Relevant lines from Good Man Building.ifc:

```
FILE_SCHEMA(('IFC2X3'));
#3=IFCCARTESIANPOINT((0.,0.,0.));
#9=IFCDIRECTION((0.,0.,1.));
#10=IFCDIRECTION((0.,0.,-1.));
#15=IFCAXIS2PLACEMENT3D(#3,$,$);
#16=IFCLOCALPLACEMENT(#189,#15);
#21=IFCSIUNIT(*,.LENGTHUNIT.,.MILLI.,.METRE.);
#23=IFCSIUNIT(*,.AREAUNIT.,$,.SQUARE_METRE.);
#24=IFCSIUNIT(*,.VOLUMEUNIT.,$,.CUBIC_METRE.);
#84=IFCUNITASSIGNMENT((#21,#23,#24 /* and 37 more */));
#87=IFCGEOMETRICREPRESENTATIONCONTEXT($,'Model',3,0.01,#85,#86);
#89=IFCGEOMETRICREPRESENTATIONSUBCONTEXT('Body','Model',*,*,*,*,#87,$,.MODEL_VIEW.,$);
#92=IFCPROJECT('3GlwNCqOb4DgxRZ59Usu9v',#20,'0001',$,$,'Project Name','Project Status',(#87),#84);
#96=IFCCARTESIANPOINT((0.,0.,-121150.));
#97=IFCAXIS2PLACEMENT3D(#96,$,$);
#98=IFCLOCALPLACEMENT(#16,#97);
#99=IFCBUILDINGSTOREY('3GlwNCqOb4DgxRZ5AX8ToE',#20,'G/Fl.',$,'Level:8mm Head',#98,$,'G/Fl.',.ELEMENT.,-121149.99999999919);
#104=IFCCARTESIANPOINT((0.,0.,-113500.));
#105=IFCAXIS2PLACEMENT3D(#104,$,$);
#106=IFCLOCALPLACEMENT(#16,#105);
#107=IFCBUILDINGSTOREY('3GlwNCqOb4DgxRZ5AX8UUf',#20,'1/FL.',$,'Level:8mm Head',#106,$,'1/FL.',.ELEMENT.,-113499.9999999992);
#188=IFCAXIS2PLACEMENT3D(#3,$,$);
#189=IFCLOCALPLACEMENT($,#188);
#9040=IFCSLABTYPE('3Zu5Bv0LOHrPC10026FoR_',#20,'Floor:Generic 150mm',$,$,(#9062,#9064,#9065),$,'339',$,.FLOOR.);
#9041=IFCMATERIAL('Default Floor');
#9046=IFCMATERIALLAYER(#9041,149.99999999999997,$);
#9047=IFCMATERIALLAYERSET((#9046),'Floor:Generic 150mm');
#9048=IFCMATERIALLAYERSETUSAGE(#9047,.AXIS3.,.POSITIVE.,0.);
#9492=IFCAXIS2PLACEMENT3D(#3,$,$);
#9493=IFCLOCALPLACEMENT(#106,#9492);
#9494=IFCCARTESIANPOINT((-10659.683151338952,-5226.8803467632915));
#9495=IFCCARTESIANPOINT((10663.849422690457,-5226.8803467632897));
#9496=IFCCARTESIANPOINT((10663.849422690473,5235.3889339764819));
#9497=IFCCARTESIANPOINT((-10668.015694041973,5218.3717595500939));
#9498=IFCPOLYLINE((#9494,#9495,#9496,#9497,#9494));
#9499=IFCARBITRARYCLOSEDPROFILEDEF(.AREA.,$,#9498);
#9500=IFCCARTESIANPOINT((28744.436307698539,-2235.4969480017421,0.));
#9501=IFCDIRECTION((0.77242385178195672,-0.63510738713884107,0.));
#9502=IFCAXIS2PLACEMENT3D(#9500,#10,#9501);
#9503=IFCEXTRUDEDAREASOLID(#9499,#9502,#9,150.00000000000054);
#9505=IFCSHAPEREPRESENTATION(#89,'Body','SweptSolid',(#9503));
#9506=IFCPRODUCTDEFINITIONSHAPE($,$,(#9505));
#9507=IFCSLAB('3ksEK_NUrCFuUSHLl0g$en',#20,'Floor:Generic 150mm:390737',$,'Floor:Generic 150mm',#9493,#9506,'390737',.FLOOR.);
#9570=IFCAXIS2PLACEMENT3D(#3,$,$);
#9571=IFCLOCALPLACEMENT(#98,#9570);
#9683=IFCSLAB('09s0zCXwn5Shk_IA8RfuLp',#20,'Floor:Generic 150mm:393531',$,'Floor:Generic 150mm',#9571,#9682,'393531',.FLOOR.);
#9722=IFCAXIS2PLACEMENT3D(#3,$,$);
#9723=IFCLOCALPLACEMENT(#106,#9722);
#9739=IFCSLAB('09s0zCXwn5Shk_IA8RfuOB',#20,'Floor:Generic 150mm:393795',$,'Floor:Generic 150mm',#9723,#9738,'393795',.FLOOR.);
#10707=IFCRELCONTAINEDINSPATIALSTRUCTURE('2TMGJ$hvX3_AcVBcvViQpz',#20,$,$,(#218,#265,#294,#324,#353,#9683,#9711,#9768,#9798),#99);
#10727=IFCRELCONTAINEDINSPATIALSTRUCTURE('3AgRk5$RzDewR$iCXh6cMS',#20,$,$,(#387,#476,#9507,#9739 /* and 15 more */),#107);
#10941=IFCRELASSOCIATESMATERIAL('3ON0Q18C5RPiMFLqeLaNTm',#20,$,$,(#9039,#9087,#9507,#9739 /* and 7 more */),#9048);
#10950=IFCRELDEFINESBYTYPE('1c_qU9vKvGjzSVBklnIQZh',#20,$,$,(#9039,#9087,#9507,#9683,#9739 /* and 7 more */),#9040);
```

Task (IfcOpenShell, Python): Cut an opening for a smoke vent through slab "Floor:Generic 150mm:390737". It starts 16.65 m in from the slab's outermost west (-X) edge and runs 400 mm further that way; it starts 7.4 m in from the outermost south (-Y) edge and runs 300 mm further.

```python
import numpy as np
import ifcopenshell
import ifcopenshell.api.feature
import ifcopenshell.api.geometry
import ifcopenshell.api.root
import ifcopenshell.geom
import ifcopenshell.util.placement
import ifcopenshell.util.representation
import ifcopenshell.util.shape
import ifcopenshell.util.unit

model = ifcopenshell.open("Good Man Building.ifc")
unit_scale = ifcopenshell.util.unit.calculate_unit_scale(model)
settings = ifcopenshell.geom.settings()


def volume(element):
    """Net volume in cubic metres, openings subtracted."""
    shape = ifcopenshell.geom.create_shape(settings, element)
    return ifcopenshell.util.shape.get_volume(shape.geometry)


slab = model.by_id(9507)
before = volume(slab)

# Extent in the slab's own axes, in metres. The edges named are its -X and -Y sides.
slab_shape = ifcopenshell.geom.create_shape(settings, slab)
vertices = ifcopenshell.util.shape.get_vertices(slab_shape.geometry)
x_min, y_min, bottom = vertices.min(axis=0)
top = vertices[:, 2].max()

opening = ifcopenshell.api.root.create_entity(model, ifc_class="IfcOpeningElement", name="Smoke vent opening")
context = ifcopenshell.util.representation.get_context(model, "Model", "Body", "MODEL_VIEW")
width, depth = 0.4, 0.3
outline = [(0.0, 0.0), (width, 0.0), (width, depth), (0.0, depth), (0.0, 0.0)]
# Overshoot both faces by 50 mm so the cut is clean.
shape = ifcopenshell.api.geometry.add_slab_representation(
    model, context=context, depth=top - bottom + 0.1, polyline=outline
)
ifcopenshell.api.geometry.assign_representation(model, product=opening, representation=shape)

matrix = ifcopenshell.util.placement.get_local_placement(slab.ObjectPlacement)
matrix[:, 3] = matrix @ np.append(np.array([x_min + 16.65, y_min + 7.4, bottom - 0.05]) / unit_scale, 1.0)
ifcopenshell.api.geometry.edit_object_placement(model, product=opening, matrix=matrix, is_si=False)
ifcopenshell.api.feature.add_feature(model, feature=opening, element=slab)

after = volume(slab)

print(f"slab volume {before:.3f} -> {after:.3f} m3")

model.write("Good Man Building_rev.ifc")
```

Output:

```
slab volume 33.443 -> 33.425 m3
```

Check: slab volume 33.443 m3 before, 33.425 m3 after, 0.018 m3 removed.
